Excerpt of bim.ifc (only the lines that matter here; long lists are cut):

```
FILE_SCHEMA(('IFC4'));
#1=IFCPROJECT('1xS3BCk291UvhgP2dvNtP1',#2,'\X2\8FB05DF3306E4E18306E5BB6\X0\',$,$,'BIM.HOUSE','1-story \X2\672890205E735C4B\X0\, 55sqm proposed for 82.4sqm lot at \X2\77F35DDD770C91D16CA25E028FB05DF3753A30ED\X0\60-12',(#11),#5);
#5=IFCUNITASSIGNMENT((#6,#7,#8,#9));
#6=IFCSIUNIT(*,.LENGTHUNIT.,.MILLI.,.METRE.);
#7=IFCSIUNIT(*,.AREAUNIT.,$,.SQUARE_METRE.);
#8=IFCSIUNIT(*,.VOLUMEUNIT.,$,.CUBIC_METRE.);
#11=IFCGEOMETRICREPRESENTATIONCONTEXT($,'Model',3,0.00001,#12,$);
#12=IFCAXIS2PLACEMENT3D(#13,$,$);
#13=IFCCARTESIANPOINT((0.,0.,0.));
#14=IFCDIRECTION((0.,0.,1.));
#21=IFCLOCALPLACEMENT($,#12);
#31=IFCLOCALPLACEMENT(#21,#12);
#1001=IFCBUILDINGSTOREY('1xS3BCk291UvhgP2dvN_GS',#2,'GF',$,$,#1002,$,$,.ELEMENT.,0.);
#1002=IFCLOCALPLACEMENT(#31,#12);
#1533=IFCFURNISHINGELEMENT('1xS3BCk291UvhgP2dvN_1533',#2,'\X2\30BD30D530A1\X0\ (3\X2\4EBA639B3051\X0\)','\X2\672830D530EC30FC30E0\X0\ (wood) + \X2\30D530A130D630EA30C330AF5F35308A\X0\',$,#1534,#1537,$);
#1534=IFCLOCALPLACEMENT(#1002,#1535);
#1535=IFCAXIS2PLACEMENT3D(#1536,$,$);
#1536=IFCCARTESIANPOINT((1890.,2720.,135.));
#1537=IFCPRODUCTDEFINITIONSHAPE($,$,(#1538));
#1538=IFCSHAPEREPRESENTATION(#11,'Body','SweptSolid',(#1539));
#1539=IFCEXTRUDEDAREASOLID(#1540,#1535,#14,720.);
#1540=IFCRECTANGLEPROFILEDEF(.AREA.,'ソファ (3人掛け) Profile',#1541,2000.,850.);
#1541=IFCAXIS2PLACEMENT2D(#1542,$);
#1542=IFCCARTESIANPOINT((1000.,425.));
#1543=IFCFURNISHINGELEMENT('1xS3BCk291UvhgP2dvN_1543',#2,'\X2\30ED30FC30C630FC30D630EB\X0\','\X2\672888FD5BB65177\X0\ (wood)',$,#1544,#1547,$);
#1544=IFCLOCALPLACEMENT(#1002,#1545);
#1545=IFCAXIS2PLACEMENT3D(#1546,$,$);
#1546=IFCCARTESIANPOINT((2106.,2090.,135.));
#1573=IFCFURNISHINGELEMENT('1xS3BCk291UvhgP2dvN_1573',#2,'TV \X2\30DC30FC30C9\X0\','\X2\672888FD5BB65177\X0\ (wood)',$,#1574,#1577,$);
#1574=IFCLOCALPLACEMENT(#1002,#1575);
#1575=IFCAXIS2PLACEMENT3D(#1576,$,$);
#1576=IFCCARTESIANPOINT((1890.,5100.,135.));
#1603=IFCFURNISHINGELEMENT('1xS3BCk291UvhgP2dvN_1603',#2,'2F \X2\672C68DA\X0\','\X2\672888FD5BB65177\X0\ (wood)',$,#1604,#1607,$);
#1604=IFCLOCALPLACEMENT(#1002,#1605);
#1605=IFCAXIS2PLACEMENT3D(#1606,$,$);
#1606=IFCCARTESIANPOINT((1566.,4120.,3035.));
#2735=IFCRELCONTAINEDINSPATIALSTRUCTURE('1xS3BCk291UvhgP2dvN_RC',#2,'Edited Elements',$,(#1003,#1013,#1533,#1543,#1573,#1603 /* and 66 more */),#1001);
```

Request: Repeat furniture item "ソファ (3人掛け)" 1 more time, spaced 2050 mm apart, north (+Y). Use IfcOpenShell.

```python
import numpy as np
import ifcopenshell
import ifcopenshell.api.geometry
import ifcopenshell.api.root
import ifcopenshell.util.element
import ifcopenshell.util.placement

model = ifcopenshell.open("bim.ifc")


def reuse_history(source, copy):
    """copy_class also copies each property set's owner history, people and application; keep the originals."""
    for rel in copy.IsDefinedBy:
        if rel.is_a("IfcRelDefinesByProperties") and (history := rel.RelatingPropertyDefinition.OwnerHistory):
            rel.RelatingPropertyDefinition.OwnerHistory = source.OwnerHistory
            ifcopenshell.util.element.remove_deep2(model, history)


source = model.by_guid("1xS3BCk291UvhgP2dvN_1533")
base = ifcopenshell.util.placement.get_local_placement(source.ObjectPlacement)
step = np.array([0.0, 1.0, 0.0]) * 2050.0

for i in range(1, 2):
    copy = ifcopenshell.api.root.copy_class(model, product=source)
    copy.Representation = ifcopenshell.util.element.copy_deep(
        model, source.Representation, exclude=["IfcGeometricRepresentationContext", "IfcRepresentationMap"]
    )
    reuse_history(source, copy)
    matrix = base.copy()
    matrix[:3, 3] += i * step
    print("added at", matrix[:3, 3].round(3) + 0.0)
    ifcopenshell.api.geometry.edit_object_placement(model, product=copy, matrix=matrix, is_si=False)

model.write("bim_v2.ifc")
```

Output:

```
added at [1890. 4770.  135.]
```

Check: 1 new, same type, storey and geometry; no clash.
